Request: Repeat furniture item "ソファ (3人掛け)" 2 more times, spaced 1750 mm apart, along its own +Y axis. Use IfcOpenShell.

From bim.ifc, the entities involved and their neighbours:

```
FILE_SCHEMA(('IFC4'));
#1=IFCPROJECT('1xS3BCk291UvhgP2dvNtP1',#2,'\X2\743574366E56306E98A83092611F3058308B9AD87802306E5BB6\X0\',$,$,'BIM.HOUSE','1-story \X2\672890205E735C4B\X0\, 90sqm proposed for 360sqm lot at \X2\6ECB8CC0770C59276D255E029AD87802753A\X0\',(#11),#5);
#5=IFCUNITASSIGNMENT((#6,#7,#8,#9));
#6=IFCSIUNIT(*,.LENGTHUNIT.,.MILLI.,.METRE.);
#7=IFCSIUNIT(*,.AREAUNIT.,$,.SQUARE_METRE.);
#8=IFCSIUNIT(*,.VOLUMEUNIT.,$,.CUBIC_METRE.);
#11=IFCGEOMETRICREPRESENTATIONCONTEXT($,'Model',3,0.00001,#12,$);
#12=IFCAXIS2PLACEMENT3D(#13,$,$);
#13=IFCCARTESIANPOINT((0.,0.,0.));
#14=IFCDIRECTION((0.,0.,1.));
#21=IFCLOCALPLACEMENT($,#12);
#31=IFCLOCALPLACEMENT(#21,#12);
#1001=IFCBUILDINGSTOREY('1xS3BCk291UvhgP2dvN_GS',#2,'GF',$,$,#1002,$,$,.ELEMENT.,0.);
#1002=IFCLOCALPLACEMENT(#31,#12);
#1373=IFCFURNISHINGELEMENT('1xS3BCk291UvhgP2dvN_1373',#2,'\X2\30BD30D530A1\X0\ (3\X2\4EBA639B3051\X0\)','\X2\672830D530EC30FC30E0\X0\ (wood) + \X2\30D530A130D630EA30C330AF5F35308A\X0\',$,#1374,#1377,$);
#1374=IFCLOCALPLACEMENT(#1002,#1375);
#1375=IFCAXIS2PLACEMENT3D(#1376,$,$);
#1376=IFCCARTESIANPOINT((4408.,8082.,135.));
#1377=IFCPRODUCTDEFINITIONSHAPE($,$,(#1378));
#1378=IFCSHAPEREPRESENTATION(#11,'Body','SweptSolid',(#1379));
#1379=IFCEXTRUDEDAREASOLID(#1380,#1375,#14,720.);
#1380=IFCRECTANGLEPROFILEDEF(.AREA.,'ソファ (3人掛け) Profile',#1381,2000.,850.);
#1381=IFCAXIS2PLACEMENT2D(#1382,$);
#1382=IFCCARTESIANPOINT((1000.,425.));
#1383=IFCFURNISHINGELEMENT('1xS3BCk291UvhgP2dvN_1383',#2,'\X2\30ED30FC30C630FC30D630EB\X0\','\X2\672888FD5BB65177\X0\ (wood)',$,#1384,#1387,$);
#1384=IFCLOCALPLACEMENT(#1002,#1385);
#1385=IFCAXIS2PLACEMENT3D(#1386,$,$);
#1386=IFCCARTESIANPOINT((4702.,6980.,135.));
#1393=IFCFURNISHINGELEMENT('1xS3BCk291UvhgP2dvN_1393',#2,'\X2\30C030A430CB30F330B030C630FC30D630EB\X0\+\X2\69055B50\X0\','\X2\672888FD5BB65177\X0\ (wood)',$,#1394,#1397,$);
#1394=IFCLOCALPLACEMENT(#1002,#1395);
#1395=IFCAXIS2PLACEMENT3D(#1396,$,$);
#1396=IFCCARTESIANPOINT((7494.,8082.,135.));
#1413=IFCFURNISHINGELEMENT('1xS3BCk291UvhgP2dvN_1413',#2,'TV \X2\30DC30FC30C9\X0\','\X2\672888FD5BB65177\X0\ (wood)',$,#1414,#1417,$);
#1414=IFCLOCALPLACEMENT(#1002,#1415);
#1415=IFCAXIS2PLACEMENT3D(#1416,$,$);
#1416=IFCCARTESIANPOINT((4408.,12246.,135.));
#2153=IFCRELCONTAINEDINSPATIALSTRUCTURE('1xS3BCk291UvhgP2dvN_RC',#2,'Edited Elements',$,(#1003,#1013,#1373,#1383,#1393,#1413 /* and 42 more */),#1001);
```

```python
import ifcopenshell
import ifcopenshell.api.geometry
import ifcopenshell.api.root
import ifcopenshell.util.element
import ifcopenshell.util.placement
import ifcopenshell.util.unit

model = ifcopenshell.open("bim.ifc")
unit_scale = ifcopenshell.util.unit.calculate_unit_scale(model)


def reuse_history(source, copy):
    """copy_class also copies each property set's owner history, people and application; keep the originals."""
    for rel in copy.IsDefinedBy:
        if rel.is_a("IfcRelDefinesByProperties") and (history := rel.RelatingPropertyDefinition.OwnerHistory):
            rel.RelatingPropertyDefinition.OwnerHistory = source.OwnerHistory
            ifcopenshell.util.element.remove_deep2(model, history)


source = model.by_id(1373)
base = ifcopenshell.util.placement.get_local_placement(source.ObjectPlacement)
step = base[:3, 1] * 1.75 / unit_scale

for i in range(1, 3):
    copy = ifcopenshell.api.root.copy_class(model, product=source)
    copy.Representation = ifcopenshell.util.element.copy_deep(
        model, source.Representation, exclude=["IfcGeometricRepresentationContext", "IfcRepresentationMap"]
    )
    reuse_history(source, copy)
    matrix = base.copy()
    matrix[:3, 3] += i * step
    print("added at", matrix[:3, 3].round(3) + 0.0)
    ifcopenshell.api.geometry.edit_object_placement(model, product=copy, matrix=matrix, is_si=False)

model.write("bim_rev.ifc")
```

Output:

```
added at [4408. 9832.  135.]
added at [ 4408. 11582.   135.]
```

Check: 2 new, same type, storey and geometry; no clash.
